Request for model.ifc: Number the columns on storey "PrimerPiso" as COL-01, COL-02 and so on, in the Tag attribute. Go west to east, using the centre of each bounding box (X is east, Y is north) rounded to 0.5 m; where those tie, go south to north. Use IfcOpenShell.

First a look at what the model holds.

```python
import ifcopenshell
import ifcopenshell.util.element
import ifcopenshell.util.placement

model = ifcopenshell.open("model.ifc")
print(model.schema)
storey = next(s for s in model.by_type("IfcBuildingStorey") if s.Name == "PrimerPiso")
columns = [e for e in ifcopenshell.util.element.get_decomposition(storey) if e.is_a("IfcColumn")]
for e in sorted(columns, key=lambda e: e.id()):
    origin = ifcopenshell.util.placement.get_local_placement(e.ObjectPlacement)[:3, 3]
    print(e.id(), e.Tag, e.Name, origin.round(2) + 0.0, sep=" | ")
```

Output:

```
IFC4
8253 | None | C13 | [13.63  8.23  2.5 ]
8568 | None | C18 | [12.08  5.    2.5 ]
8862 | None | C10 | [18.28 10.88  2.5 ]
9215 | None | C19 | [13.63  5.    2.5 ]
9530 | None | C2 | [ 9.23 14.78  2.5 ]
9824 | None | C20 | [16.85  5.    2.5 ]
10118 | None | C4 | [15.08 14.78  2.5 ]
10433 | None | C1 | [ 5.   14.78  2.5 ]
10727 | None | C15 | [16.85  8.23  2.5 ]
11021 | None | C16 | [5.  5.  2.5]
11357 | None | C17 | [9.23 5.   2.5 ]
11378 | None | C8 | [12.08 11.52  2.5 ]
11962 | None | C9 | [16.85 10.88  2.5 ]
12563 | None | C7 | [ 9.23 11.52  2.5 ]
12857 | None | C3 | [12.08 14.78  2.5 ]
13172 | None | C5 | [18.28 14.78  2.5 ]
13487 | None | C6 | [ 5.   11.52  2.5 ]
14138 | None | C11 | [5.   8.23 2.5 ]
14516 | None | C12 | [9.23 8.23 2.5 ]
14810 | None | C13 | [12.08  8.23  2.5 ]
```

```python
import ifcopenshell
import ifcopenshell.geom
import ifcopenshell.util.element
import ifcopenshell.util.shape

model = ifcopenshell.open("model.ifc")
settings = ifcopenshell.geom.settings()
settings.set("use-world-coords", True)


def centre(element):
    shape = ifcopenshell.geom.create_shape(settings, element)
    return ifcopenshell.util.shape.get_bbox_centroid(shape.geometry)


storey = next(s for s in model.by_type("IfcBuildingStorey") if s.Name == "PrimerPiso")
columns = [e for e in ifcopenshell.util.element.get_decomposition(storey) if e.is_a("IfcColumn")]

# Insertion points can sit at a corner or the storey origin, so sort by the geometry (in metres).
centres = {e: centre(e) for e in columns}
columns.sort(key=lambda e: (round(centres[e][0] / 0.5), centres[e][1]))

for i, e in enumerate(columns, start=1):
    number = f"COL-{i:02d}"
    e.Tag = number
    print(e.id(), number)

model.write("model_updated.ifc")
```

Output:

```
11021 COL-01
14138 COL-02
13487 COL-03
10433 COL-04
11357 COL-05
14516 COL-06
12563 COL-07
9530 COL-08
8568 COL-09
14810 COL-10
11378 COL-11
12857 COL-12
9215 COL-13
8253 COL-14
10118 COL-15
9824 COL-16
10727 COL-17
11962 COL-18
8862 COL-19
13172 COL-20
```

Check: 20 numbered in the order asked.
